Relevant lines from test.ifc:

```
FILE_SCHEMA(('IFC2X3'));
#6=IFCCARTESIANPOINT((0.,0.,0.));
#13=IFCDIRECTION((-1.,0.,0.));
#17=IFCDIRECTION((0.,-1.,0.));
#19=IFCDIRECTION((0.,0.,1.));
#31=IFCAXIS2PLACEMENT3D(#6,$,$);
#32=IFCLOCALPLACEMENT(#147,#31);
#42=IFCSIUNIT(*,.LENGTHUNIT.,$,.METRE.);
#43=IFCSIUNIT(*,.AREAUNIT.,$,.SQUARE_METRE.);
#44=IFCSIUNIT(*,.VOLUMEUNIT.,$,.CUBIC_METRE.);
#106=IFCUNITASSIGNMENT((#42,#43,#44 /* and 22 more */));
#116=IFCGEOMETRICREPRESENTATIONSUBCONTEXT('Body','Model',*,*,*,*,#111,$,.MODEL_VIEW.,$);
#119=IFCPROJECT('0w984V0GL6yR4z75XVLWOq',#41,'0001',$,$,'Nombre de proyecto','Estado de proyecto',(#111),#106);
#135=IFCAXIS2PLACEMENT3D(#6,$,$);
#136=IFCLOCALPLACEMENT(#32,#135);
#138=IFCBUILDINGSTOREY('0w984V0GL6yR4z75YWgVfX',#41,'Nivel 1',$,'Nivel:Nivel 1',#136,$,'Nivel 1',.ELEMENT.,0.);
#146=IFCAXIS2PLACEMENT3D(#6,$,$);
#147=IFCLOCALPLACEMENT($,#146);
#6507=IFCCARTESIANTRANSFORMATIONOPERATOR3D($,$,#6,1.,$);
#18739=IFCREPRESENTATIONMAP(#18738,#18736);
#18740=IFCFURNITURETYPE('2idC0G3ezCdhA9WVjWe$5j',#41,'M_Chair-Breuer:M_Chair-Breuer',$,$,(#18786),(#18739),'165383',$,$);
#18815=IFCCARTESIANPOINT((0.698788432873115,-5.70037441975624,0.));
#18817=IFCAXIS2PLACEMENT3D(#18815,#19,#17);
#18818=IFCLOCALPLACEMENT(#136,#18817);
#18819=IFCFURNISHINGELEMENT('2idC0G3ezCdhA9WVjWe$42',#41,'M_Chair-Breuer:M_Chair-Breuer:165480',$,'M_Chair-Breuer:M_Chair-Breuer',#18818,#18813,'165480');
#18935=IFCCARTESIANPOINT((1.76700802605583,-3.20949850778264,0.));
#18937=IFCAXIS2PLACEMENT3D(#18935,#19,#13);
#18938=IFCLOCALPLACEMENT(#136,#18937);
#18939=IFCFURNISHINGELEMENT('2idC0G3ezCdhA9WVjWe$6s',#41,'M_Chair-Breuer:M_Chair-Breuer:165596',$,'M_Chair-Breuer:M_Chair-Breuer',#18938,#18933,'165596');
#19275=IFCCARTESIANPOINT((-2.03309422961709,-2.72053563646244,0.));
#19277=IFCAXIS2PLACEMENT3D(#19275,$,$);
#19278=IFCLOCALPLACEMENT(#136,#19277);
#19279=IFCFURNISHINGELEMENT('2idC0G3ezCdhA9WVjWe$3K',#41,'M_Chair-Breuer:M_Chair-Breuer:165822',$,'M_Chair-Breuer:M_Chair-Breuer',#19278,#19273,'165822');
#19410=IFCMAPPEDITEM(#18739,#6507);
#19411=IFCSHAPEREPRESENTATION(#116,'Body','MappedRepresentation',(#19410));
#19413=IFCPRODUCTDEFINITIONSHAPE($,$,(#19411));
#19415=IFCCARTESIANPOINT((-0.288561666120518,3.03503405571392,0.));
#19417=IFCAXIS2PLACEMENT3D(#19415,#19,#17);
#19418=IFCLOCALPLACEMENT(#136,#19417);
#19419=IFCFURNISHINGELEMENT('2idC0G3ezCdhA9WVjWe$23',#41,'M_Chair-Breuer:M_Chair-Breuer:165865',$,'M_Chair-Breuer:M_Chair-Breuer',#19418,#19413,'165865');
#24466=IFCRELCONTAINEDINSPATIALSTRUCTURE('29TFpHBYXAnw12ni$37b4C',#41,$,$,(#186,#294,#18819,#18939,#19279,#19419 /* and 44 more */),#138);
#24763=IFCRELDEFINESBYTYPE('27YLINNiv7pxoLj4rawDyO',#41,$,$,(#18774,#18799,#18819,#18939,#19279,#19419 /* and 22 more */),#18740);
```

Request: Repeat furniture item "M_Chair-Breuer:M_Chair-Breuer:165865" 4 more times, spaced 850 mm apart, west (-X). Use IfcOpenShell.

```python
import numpy as np
import ifcopenshell
import ifcopenshell.api.geometry
import ifcopenshell.api.root
import ifcopenshell.util.element
import ifcopenshell.util.placement

model = ifcopenshell.open("test.ifc")


def reuse_history(source, copy):
    """copy_class also copies each property set's owner history, people and application; keep the originals."""
    for rel in copy.IsDefinedBy:
        if rel.is_a("IfcRelDefinesByProperties") and (history := rel.RelatingPropertyDefinition.OwnerHistory):
            rel.RelatingPropertyDefinition.OwnerHistory = source.OwnerHistory
            ifcopenshell.util.element.remove_deep2(model, history)


source = model.by_id(19419)
base = ifcopenshell.util.placement.get_local_placement(source.ObjectPlacement)
step = np.array([-1.0, 0.0, 0.0]) * 0.85

for i in range(1, 5):
    copy = ifcopenshell.api.root.copy_class(model, product=source)
    copy.Representation = ifcopenshell.util.element.copy_deep(
        model, source.Representation, exclude=["IfcGeometricRepresentationContext", "IfcRepresentationMap"]
    )
    copy.Name = "M_Chair-Breuer:M_Chair-Breuer"
    copy.Tag = None
    reuse_history(source, copy)
    matrix = base.copy()
    matrix[:3, 3] += i * step
    print("added at", matrix[:3, 3].round(3) + 0.0)
    ifcopenshell.api.geometry.edit_object_placement(model, product=copy, matrix=matrix, is_si=False)

model.write("test_edited.ifc")
```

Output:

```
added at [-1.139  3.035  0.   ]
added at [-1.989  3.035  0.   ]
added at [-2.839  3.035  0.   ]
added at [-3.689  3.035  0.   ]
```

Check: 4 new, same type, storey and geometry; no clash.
